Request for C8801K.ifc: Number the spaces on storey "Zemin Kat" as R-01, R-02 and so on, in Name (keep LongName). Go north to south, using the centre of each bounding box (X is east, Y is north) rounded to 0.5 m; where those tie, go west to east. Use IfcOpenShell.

First a look at what the model holds.

```python
import ifcopenshell
import ifcopenshell.util.element
import ifcopenshell.util.placement

model = ifcopenshell.open("C8801K.ifc")
print(model.schema)
storey = next(s for s in model.by_type("IfcBuildingStorey") if s.Name == "Zemin Kat")
spaces = [e for e in ifcopenshell.util.element.get_decomposition(storey) if e.is_a("IfcSpace")]
for e in sorted(spaces, key=lambda e: e.id()):
    origin = ifcopenshell.util.placement.get_local_placement(e.ObjectPlacement)[:3, 3]
    print(e.id(), e.Name, e.LongName, origin.round(2) + 0.0, sep=" | ")
```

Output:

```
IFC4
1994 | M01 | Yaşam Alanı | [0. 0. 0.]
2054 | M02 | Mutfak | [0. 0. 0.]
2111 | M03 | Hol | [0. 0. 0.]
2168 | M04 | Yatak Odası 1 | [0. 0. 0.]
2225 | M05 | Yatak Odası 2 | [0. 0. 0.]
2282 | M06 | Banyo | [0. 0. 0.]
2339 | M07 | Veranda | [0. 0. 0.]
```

```python
import ifcopenshell
import ifcopenshell.geom
import ifcopenshell.util.element
import ifcopenshell.util.shape

model = ifcopenshell.open("C8801K.ifc")
settings = ifcopenshell.geom.settings()
settings.set("use-world-coords", True)


def centre(element):
    shape = ifcopenshell.geom.create_shape(settings, element)
    return ifcopenshell.util.shape.get_bbox_centroid(shape.geometry)


storey = next(s for s in model.by_type("IfcBuildingStorey") if s.Name == "Zemin Kat")
spaces = [e for e in ifcopenshell.util.element.get_decomposition(storey) if e.is_a("IfcSpace")]

# Insertion points can sit at a corner or the storey origin, so sort by the geometry (in metres).
centres = {e: centre(e) for e in spaces}
spaces.sort(key=lambda e: (-round(centres[e][1] / 0.5), centres[e][0]))

for i, e in enumerate(spaces, start=1):
    number = f"R-{i:02d}"
    e.Name = number
    print(e.id(), number)

model.write("C8801K-out.ifc")
```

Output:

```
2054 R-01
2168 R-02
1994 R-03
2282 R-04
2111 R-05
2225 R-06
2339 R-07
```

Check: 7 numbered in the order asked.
